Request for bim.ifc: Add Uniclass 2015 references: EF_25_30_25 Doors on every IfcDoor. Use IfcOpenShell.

First a look at what the model holds.

```python
import ifcopenshell

model = ifcopenshell.open("bim.ifc")
print(model.schema)
print("classifications:", [c.Name for c in model.by_type("IfcClassification")])
for ifc_class in ("IfcDoor", "IfcRoof", "IfcStair", "IfcWall", "IfcWindow"):
    print(ifc_class, len(model.by_type(ifc_class)))
```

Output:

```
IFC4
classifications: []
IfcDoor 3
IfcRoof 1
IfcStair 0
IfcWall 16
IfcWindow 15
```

```python
import ifcopenshell
import ifcopenshell.api.classification

model = ifcopenshell.open("bim.ifc")

system = ifcopenshell.api.classification.add_classification(model, classification="Uniclass 2015")

codes = {
    "IfcDoor": ("EF_25_30_25", "Doors"),
}
for ifc_class, (code, name) in codes.items():
    products = model.by_type(ifc_class)
    ifcopenshell.api.classification.add_reference(
        model, products=products, classification=system, identification=code, name=name
    )
    print(code, len(products))

model.write("bim_v2.ifc")
```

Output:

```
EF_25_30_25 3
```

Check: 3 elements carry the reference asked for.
